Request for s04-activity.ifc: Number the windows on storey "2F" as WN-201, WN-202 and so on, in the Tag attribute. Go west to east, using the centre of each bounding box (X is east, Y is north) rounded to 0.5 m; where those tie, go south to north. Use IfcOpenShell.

First a look at what the model holds.

```python
import ifcopenshell
import ifcopenshell.util.element
import ifcopenshell.util.placement

model = ifcopenshell.open("s04-activity.ifc")
print(model.schema)
storey = next(s for s in model.by_type("IfcBuildingStorey") if s.Name == "2F")
windows = [e for e in ifcopenshell.util.element.get_decomposition(storey) if e.is_a("IfcWindow")]
for e in sorted(windows, key=lambda e: e.id()):
    origin = ifcopenshell.util.placement.get_local_placement(e.ObjectPlacement)[:3, 3]
    print(e.id(), e.Tag, e.Name, origin.round(2) + 0.0, sep=" | ")
```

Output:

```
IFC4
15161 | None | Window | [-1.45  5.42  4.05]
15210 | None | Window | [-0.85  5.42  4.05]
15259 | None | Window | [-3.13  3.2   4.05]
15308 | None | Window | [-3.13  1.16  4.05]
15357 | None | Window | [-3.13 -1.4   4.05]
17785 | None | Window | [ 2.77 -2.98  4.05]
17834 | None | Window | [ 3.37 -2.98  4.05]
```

```python
import ifcopenshell
import ifcopenshell.geom
import ifcopenshell.util.element
import ifcopenshell.util.shape

model = ifcopenshell.open("s04-activity.ifc")
settings = ifcopenshell.geom.settings()
settings.set("use-world-coords", True)


def centre(element):
    shape = ifcopenshell.geom.create_shape(settings, element)
    return ifcopenshell.util.shape.get_bbox_centroid(shape.geometry)


storey = next(s for s in model.by_type("IfcBuildingStorey") if s.Name == "2F")
windows = [e for e in ifcopenshell.util.element.get_decomposition(storey) if e.is_a("IfcWindow")]

# Insertion points can sit at a corner or the storey origin, so sort by the geometry (in metres).
centres = {e: centre(e) for e in windows}
windows.sort(key=lambda e: (round(centres[e][0] / 0.5), centres[e][1]))

for i, e in enumerate(windows, start=1):
    number = f"WN-2{i:02d}"
    e.Tag = number
    print(e.id(), number)

model.write("s04-activity-out.ifc")
```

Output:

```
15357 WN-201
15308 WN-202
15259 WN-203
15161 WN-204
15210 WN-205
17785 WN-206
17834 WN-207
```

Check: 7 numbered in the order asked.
